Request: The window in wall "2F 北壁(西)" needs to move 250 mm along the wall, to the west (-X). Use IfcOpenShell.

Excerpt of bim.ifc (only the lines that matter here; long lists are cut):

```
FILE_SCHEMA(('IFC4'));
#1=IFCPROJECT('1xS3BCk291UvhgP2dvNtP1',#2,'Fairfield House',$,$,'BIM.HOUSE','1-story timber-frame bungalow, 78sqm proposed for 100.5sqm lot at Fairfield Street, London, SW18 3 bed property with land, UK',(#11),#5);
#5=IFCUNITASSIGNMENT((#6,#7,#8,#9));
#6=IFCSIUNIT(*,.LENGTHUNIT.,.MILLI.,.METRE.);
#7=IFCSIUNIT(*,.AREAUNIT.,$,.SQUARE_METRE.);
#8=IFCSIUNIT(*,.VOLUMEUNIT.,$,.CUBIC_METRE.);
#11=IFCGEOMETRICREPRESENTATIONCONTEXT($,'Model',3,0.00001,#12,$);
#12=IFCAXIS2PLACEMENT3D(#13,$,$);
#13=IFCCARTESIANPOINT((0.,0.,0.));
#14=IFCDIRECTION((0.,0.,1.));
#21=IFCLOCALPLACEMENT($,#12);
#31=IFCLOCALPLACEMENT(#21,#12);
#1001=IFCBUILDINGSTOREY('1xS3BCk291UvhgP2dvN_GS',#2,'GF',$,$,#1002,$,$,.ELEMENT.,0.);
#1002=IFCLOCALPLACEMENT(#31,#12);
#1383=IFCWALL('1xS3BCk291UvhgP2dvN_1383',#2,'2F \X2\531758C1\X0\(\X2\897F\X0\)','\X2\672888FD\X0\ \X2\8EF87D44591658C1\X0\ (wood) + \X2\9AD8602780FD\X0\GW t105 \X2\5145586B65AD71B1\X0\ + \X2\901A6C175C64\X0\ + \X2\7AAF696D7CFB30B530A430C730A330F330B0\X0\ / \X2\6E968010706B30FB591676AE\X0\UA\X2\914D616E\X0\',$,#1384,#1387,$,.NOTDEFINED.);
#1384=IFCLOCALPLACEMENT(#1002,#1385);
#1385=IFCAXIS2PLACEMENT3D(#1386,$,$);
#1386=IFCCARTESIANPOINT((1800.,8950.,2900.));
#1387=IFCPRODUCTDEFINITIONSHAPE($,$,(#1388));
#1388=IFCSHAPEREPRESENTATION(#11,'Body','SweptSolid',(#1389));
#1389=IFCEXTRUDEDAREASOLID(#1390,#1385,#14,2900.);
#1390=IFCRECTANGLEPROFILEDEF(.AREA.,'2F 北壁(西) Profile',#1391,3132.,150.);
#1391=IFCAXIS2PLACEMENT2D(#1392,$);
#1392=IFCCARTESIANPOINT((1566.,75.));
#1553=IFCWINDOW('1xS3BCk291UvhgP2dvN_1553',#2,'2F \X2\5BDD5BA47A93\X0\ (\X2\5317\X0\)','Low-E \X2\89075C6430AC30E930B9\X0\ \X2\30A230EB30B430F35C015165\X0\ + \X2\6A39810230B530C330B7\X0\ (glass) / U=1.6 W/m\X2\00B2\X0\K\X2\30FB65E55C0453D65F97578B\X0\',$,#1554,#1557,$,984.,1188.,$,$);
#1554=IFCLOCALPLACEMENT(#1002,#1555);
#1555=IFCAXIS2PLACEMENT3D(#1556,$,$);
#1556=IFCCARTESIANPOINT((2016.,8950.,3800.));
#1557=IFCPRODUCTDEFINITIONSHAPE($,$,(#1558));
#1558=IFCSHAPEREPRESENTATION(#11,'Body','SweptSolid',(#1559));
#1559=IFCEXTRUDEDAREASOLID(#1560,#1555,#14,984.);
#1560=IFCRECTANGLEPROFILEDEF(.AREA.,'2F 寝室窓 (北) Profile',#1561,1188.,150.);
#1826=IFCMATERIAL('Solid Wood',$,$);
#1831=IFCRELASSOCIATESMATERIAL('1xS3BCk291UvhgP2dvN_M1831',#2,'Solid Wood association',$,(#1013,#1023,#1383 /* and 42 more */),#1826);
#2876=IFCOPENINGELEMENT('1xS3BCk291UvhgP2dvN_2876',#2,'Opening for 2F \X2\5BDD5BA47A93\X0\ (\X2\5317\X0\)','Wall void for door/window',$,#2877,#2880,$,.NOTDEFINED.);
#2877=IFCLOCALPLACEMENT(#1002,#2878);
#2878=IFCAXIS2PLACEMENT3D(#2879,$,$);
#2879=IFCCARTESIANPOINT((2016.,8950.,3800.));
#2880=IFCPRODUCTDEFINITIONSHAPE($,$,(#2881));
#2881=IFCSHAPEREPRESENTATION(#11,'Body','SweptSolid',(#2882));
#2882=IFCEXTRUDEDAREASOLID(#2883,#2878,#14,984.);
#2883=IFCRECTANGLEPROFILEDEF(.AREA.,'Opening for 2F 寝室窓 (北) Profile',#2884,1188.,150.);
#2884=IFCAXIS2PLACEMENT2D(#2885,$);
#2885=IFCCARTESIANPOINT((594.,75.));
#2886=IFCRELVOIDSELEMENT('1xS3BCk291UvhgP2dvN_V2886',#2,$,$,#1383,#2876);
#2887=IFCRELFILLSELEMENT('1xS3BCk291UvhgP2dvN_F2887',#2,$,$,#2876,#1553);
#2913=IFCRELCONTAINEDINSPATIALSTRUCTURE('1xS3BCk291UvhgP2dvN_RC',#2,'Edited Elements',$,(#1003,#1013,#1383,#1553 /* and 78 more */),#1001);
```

```python
import ifcopenshell
import ifcopenshell.api.geometry
import ifcopenshell.util.placement
import ifcopenshell.util.unit

model = ifcopenshell.open("bim.ifc")
unit_scale = ifcopenshell.util.unit.calculate_unit_scale(model)

window = model.by_guid("1xS3BCk291UvhgP2dvN_1553")
opening = window.FillsVoids[0].RelatingOpeningElement
wall = opening.VoidsElements[0].RelatingBuildingElement

wall_matrix = ifcopenshell.util.placement.get_local_placement(wall.ObjectPlacement)
shift = wall_matrix[:3, 0] * -0.25 / unit_scale
before = ifcopenshell.util.placement.get_local_placement(window.ObjectPlacement)[:3, 3].copy()

# The window is not placed relative to its opening, so move both.
for product in (opening, window):
    matrix = ifcopenshell.util.placement.get_local_placement(product.ObjectPlacement)
    matrix[:3, 3] += shift
    ifcopenshell.api.geometry.edit_object_placement(model, product=product, matrix=matrix, is_si=False)

after = ifcopenshell.util.placement.get_local_placement(window.ObjectPlacement)[:3, 3]
print("window moved by", (after - before).round(3) + 0.0)

model.write("bim_edited.ifc")
```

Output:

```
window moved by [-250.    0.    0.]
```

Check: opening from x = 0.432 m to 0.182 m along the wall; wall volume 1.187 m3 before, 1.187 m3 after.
